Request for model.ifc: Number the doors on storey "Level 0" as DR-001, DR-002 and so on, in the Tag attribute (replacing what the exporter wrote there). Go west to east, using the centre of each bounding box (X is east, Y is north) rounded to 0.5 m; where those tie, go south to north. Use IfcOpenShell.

First a look at what the model holds.

```python
import ifcopenshell
import ifcopenshell.util.element
import ifcopenshell.util.placement

model = ifcopenshell.open("model.ifc")
print(model.schema)
storey = next(s for s in model.by_type("IfcBuildingStorey") if s.Name == "Level 0")
doors = [e for e in ifcopenshell.util.element.get_decomposition(storey) if e.is_a("IfcDoor")]
for e in sorted(doors, key=lambda e: e.id()):
    origin = ifcopenshell.util.placement.get_local_placement(e.ObjectPlacement)[:3, 3]
    print(e.id(), e.Tag, e.Name, origin.round(2) + 0.0, sep=" | ")
```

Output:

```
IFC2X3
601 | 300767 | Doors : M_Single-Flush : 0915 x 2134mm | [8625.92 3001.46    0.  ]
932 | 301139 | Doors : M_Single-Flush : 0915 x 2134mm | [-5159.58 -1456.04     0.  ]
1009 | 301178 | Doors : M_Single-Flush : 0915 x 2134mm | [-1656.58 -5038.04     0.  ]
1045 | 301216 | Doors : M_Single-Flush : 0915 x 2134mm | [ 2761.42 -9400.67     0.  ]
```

```python
import ifcopenshell
import ifcopenshell.geom
import ifcopenshell.util.element
import ifcopenshell.util.shape

model = ifcopenshell.open("model.ifc")
settings = ifcopenshell.geom.settings()
settings.set("use-world-coords", True)


def centre(element):
    shape = ifcopenshell.geom.create_shape(settings, element)
    return ifcopenshell.util.shape.get_bbox_centroid(shape.geometry)


storey = next(s for s in model.by_type("IfcBuildingStorey") if s.Name == "Level 0")
doors = [e for e in ifcopenshell.util.element.get_decomposition(storey) if e.is_a("IfcDoor")]

# Insertion points can sit at a corner or the storey origin, so sort by the geometry (in metres).
centres = {e: centre(e) for e in doors}
doors.sort(key=lambda e: (round(centres[e][0] / 0.5), centres[e][1]))

for i, e in enumerate(doors, start=1):
    number = f"DR-0{i:02d}"
    e.Tag = number
    print(e.id(), number)

model.write("model_updated.ifc")
```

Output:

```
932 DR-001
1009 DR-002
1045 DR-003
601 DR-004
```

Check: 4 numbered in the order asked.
